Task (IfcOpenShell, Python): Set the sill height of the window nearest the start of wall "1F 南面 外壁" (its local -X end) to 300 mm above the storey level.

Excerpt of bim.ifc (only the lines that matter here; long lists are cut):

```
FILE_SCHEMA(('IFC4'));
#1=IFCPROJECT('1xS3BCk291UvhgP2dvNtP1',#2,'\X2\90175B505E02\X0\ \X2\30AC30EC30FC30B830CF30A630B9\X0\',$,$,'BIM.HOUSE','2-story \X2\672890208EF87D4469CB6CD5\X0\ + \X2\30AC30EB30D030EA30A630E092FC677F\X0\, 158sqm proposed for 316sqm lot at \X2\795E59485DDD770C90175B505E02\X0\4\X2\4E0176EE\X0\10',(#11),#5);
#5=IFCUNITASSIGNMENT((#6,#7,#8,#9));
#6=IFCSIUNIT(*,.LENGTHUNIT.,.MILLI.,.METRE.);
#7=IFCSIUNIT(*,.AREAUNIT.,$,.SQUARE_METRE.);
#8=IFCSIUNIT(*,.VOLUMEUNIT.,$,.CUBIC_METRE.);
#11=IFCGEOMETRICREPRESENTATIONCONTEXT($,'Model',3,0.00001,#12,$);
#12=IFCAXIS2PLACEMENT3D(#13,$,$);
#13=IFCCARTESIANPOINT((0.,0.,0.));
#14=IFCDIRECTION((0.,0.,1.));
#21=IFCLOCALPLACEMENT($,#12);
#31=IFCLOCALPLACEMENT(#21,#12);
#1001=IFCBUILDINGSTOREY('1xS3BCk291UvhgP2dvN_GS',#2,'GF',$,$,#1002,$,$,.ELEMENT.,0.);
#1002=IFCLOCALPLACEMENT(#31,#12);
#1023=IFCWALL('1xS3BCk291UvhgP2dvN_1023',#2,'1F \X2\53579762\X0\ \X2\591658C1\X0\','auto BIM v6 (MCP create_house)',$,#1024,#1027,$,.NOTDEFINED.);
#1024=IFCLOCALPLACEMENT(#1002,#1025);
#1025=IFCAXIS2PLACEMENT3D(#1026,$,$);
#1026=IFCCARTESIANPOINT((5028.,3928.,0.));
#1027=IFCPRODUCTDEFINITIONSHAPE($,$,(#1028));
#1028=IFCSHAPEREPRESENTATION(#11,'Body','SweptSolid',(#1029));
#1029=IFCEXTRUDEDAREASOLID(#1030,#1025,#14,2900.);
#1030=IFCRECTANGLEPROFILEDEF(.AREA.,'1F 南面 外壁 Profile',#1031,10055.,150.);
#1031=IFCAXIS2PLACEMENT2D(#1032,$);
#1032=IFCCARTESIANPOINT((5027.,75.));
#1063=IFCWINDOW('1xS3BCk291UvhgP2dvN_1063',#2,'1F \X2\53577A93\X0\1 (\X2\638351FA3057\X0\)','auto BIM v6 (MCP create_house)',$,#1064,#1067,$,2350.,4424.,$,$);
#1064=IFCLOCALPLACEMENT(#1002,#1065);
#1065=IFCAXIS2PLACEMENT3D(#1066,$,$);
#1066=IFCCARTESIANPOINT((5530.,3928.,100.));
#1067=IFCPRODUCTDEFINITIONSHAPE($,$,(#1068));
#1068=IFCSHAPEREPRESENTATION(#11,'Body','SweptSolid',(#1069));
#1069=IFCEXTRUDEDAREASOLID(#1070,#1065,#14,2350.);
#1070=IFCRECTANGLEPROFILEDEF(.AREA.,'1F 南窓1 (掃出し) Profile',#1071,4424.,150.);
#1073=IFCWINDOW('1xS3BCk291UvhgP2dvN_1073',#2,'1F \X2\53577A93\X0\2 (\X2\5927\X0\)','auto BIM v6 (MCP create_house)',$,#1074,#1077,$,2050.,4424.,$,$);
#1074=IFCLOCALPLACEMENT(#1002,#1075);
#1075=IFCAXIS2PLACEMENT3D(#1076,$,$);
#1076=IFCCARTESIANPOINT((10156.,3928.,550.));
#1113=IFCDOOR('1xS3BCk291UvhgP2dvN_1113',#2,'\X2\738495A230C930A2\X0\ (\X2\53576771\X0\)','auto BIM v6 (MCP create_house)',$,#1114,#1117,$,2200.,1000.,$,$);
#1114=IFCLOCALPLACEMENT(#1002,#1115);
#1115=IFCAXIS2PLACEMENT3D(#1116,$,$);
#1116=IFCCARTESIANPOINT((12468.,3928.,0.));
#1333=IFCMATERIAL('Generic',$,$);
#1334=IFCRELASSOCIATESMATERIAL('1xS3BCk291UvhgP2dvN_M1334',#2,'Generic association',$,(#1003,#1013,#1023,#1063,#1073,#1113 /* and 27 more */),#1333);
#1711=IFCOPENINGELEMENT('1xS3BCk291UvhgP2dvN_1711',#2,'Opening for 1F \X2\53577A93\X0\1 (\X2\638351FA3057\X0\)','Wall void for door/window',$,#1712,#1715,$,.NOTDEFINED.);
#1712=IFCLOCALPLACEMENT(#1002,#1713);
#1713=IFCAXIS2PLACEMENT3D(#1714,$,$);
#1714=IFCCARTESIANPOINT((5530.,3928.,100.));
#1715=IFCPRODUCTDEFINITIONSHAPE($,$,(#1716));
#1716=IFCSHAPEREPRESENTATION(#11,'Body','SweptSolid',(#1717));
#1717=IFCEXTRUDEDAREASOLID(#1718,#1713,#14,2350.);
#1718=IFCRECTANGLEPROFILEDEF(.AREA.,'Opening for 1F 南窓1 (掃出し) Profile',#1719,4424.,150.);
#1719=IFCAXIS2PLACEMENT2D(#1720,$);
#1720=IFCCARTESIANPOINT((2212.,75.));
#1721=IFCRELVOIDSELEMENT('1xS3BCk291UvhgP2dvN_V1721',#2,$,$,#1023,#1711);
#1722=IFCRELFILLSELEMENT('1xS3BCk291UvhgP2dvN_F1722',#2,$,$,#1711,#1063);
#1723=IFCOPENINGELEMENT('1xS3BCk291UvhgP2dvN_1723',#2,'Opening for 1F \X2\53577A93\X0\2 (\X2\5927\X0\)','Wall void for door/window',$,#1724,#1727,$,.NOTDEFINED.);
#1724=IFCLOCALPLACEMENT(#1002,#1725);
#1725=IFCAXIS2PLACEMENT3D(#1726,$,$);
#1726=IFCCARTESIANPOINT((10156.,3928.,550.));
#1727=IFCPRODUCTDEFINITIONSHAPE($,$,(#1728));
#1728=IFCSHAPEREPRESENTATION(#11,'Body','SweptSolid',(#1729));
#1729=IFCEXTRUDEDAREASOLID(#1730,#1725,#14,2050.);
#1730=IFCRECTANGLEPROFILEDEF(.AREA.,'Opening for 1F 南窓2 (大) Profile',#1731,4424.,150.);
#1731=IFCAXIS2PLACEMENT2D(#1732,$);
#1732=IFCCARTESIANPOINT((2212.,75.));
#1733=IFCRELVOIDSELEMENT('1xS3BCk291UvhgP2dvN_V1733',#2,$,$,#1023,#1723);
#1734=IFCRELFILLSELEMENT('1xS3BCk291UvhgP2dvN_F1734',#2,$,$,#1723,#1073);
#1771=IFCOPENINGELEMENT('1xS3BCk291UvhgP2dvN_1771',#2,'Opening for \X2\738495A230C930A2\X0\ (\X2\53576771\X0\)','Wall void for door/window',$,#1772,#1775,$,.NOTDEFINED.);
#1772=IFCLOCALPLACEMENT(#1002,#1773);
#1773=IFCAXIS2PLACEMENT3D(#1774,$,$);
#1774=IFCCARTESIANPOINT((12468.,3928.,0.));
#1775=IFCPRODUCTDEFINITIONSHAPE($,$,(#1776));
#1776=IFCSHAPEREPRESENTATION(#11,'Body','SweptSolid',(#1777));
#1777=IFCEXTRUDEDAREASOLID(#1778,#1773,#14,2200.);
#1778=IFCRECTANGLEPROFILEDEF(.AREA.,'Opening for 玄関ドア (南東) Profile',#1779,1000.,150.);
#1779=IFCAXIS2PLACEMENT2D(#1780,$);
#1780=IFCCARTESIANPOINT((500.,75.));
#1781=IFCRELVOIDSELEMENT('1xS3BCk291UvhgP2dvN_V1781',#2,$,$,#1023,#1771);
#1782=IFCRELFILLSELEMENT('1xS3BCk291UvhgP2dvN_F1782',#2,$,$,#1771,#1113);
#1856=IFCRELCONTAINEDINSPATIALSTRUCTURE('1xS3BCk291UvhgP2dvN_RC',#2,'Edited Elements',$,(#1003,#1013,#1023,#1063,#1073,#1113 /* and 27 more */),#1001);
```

```python
import numpy as np
import ifcopenshell
import ifcopenshell.api.geometry
import ifcopenshell.geom
import ifcopenshell.util.element
import ifcopenshell.util.placement
import ifcopenshell.util.shape
import ifcopenshell.util.unit

model = ifcopenshell.open("bim.ifc")
unit_scale = ifcopenshell.util.unit.calculate_unit_scale(model)

window = model.by_guid("1xS3BCk291UvhgP2dvN_1063")
opening = window.FillsVoids[0].RelatingOpeningElement
storey = ifcopenshell.util.element.get_container(window, ifc_class="IfcBuildingStorey")
level = ifcopenshell.util.placement.get_local_placement(storey.ObjectPlacement)[2, 3]

# The opening's origin need not be at the sill, so measure its lowest point.
shape = ifcopenshell.geom.create_shape(ifcopenshell.geom.settings(), opening)
bottom = ifcopenshell.util.shape.get_shape_bottom_elevation(shape, shape.geometry) / unit_scale
dz = level + 0.3 / unit_scale - bottom

shift = np.array([0.0, 0.0, dz])
# The window is not placed relative to its opening, so move both.
for product in (opening, window):
    matrix = ifcopenshell.util.placement.get_local_placement(product.ObjectPlacement)
    matrix[:3, 3] += shift
    ifcopenshell.api.geometry.edit_object_placement(model, product=product, matrix=matrix, is_si=False)

print(f"moved by {dz * unit_scale:+.3f} m")

model.write("bim_v2.ifc")
```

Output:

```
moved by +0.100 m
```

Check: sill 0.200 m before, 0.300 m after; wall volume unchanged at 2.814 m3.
